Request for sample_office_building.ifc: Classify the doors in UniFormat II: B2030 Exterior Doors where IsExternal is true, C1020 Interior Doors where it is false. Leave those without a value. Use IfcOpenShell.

First a look at what the model holds.

```python
import ifcopenshell
import ifcopenshell.util.element

model = ifcopenshell.open("sample_office_building.ifc")
print(model.schema)
print("classifications:", [c.Name for c in model.by_type("IfcClassification")])
values = [ifcopenshell.util.element.get_pset(e, "Pset_DoorCommon", "IsExternal") for e in model.by_type("IfcDoor")]
for value in (True, False, None):
    print("IsExternal", value, values.count(value))
```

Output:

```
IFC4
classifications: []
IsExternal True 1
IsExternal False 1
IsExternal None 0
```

```python
import ifcopenshell
import ifcopenshell.api.classification
import ifcopenshell.util.element

model = ifcopenshell.open("sample_office_building.ifc")

system = ifcopenshell.api.classification.add_classification(model, classification="UniFormat II")

doors = model.by_type("IfcDoor")
external = {e: ifcopenshell.util.element.get_pset(e, "Pset_DoorCommon", "IsExternal") for e in doors}
for flag, code, name in ((True, "B2030", "Exterior Doors"), (False, "C1020", "Interior Doors")):
    products = [e for e in doors if external[e] is flag]
    ifcopenshell.api.classification.add_reference(
        model, products=products, classification=system, identification=code, name=name
    )
    print(code, len(products))

model.write("sample_office_building_rev.ifc")
```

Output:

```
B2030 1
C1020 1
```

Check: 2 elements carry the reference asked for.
